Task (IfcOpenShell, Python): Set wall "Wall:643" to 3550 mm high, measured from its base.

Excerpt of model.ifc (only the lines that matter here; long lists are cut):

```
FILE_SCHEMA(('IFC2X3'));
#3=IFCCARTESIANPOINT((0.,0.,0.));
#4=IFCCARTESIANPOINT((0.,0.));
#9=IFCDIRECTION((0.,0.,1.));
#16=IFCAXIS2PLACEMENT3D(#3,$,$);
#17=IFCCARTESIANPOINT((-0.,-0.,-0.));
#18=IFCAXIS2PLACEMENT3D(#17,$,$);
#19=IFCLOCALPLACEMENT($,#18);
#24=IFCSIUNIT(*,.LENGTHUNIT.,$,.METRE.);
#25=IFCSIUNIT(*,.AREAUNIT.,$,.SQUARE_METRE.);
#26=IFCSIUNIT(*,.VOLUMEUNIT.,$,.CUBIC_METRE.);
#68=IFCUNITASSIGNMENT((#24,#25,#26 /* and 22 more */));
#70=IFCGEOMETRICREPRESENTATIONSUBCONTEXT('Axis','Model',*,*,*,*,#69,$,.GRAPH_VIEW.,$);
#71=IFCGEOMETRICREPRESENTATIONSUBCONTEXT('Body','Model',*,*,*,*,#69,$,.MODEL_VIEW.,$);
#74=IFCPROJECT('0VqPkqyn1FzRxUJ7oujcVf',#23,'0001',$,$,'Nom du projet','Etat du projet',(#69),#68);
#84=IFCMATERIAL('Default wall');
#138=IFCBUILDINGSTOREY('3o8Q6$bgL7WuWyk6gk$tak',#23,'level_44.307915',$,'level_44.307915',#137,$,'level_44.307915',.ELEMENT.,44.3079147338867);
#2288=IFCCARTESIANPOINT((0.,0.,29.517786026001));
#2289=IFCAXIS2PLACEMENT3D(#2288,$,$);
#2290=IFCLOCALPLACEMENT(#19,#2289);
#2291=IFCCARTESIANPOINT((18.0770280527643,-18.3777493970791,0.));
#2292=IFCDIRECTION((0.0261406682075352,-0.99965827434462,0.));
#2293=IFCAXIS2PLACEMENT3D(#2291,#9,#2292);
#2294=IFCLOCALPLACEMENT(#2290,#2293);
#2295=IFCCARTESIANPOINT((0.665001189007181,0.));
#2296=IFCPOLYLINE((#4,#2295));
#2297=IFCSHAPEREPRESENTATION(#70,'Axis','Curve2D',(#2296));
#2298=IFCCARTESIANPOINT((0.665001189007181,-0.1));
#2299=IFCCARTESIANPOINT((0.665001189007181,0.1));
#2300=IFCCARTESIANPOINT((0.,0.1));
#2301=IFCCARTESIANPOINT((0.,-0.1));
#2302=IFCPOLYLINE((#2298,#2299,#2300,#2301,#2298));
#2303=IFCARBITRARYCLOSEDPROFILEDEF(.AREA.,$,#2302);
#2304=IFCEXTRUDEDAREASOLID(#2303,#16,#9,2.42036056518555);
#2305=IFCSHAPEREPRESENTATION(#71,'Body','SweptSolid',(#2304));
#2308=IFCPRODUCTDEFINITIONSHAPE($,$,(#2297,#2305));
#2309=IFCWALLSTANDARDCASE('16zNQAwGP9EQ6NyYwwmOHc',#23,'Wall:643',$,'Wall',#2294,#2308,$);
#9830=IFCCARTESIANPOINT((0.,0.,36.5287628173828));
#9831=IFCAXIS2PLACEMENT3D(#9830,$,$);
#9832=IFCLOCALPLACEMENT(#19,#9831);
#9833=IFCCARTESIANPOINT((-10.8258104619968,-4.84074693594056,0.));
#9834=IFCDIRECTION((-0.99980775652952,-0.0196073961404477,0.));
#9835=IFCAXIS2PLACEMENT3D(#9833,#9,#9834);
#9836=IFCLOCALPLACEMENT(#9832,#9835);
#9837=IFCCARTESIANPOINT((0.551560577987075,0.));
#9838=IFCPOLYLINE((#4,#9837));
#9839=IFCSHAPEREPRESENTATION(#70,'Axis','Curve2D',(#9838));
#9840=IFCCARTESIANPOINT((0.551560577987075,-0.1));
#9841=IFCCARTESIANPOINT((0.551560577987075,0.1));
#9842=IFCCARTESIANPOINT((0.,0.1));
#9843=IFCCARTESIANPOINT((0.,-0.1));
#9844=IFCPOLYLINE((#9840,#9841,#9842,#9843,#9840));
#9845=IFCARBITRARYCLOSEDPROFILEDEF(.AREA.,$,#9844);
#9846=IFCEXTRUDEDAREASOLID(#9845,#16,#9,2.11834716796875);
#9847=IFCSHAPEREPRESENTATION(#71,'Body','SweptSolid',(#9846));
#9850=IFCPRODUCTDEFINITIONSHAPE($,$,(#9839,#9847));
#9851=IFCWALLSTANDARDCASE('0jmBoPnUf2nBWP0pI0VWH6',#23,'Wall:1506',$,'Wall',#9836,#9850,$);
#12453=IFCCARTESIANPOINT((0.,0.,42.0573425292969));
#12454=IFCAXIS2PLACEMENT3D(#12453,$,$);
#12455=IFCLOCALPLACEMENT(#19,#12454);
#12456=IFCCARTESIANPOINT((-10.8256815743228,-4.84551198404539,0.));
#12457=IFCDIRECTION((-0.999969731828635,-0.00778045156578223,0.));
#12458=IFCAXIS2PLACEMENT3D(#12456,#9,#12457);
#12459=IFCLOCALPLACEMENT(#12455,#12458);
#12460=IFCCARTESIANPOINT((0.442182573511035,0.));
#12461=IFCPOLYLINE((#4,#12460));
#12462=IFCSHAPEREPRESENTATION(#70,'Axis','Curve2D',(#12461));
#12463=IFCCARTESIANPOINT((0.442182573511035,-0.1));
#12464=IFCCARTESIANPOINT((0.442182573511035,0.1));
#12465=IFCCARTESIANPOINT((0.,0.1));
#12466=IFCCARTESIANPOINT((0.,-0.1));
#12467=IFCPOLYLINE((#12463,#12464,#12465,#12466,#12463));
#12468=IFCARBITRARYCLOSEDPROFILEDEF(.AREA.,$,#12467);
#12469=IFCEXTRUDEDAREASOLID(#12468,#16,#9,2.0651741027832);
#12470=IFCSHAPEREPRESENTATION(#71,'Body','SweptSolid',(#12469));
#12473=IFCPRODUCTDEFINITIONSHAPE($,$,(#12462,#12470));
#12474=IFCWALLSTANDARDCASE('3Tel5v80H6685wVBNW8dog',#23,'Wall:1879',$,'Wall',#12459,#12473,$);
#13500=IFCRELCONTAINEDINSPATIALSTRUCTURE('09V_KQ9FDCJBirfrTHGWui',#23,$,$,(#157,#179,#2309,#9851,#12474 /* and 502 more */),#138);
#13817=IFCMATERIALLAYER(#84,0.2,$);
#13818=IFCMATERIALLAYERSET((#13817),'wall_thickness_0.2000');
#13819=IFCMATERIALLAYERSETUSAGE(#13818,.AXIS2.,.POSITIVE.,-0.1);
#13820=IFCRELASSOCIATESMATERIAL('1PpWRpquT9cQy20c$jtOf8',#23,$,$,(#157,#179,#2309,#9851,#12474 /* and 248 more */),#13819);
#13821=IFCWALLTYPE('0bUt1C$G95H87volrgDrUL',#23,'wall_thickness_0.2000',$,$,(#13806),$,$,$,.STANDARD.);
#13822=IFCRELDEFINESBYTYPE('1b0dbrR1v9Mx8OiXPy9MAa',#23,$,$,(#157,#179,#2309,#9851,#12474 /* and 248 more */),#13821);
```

```python
import ifcopenshell
import ifcopenshell.geom
import ifcopenshell.util.representation
import ifcopenshell.util.shape
import ifcopenshell.util.unit

model = ifcopenshell.open("model.ifc")
unit_scale = ifcopenshell.util.unit.calculate_unit_scale(model)
settings = ifcopenshell.geom.settings()


def volume(element):
    """Net volume in cubic metres, openings subtracted."""
    shape = ifcopenshell.geom.create_shape(settings, element)
    return ifcopenshell.util.shape.get_volume(shape.geometry)


wall = model.by_guid("16zNQAwGP9EQ6NyYwwmOHc")
before = volume(wall)

body = ifcopenshell.util.representation.get_representation(wall, "Model", "Body")
solid = body.Items[0]
old_height = solid.Depth
solid.Depth = 3.55 / unit_scale
after = volume(wall)

print(f"height {old_height:g} -> {solid.Depth:g}, volume {before:.3f} -> {after:.3f} m3")

model.write("model_edited.ifc")
```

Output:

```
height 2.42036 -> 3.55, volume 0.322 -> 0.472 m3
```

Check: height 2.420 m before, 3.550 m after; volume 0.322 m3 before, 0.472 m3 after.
